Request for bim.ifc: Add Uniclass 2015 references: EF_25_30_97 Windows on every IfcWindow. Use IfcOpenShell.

First a look at what the model holds.

```python
import ifcopenshell

model = ifcopenshell.open("bim.ifc")
print(model.schema)
print("classifications:", [c.Name for c in model.by_type("IfcClassification")])
for ifc_class in ("IfcDoor", "IfcRoof", "IfcStair", "IfcWall", "IfcWindow"):
    print(ifc_class, len(model.by_type(ifc_class)))
```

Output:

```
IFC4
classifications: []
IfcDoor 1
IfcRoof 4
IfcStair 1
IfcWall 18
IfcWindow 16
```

```python
import ifcopenshell
import ifcopenshell.api.classification

model = ifcopenshell.open("bim.ifc")

system = ifcopenshell.api.classification.add_classification(model, classification="Uniclass 2015")

codes = {
    "IfcWindow": ("EF_25_30_97", "Windows"),
}
for ifc_class, (code, name) in codes.items():
    products = model.by_type(ifc_class)
    ifcopenshell.api.classification.add_reference(
        model, products=products, classification=system, identification=code, name=name
    )
    print(code, len(products))

model.write("bim_edited.ifc")
```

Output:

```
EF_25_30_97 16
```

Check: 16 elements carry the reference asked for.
